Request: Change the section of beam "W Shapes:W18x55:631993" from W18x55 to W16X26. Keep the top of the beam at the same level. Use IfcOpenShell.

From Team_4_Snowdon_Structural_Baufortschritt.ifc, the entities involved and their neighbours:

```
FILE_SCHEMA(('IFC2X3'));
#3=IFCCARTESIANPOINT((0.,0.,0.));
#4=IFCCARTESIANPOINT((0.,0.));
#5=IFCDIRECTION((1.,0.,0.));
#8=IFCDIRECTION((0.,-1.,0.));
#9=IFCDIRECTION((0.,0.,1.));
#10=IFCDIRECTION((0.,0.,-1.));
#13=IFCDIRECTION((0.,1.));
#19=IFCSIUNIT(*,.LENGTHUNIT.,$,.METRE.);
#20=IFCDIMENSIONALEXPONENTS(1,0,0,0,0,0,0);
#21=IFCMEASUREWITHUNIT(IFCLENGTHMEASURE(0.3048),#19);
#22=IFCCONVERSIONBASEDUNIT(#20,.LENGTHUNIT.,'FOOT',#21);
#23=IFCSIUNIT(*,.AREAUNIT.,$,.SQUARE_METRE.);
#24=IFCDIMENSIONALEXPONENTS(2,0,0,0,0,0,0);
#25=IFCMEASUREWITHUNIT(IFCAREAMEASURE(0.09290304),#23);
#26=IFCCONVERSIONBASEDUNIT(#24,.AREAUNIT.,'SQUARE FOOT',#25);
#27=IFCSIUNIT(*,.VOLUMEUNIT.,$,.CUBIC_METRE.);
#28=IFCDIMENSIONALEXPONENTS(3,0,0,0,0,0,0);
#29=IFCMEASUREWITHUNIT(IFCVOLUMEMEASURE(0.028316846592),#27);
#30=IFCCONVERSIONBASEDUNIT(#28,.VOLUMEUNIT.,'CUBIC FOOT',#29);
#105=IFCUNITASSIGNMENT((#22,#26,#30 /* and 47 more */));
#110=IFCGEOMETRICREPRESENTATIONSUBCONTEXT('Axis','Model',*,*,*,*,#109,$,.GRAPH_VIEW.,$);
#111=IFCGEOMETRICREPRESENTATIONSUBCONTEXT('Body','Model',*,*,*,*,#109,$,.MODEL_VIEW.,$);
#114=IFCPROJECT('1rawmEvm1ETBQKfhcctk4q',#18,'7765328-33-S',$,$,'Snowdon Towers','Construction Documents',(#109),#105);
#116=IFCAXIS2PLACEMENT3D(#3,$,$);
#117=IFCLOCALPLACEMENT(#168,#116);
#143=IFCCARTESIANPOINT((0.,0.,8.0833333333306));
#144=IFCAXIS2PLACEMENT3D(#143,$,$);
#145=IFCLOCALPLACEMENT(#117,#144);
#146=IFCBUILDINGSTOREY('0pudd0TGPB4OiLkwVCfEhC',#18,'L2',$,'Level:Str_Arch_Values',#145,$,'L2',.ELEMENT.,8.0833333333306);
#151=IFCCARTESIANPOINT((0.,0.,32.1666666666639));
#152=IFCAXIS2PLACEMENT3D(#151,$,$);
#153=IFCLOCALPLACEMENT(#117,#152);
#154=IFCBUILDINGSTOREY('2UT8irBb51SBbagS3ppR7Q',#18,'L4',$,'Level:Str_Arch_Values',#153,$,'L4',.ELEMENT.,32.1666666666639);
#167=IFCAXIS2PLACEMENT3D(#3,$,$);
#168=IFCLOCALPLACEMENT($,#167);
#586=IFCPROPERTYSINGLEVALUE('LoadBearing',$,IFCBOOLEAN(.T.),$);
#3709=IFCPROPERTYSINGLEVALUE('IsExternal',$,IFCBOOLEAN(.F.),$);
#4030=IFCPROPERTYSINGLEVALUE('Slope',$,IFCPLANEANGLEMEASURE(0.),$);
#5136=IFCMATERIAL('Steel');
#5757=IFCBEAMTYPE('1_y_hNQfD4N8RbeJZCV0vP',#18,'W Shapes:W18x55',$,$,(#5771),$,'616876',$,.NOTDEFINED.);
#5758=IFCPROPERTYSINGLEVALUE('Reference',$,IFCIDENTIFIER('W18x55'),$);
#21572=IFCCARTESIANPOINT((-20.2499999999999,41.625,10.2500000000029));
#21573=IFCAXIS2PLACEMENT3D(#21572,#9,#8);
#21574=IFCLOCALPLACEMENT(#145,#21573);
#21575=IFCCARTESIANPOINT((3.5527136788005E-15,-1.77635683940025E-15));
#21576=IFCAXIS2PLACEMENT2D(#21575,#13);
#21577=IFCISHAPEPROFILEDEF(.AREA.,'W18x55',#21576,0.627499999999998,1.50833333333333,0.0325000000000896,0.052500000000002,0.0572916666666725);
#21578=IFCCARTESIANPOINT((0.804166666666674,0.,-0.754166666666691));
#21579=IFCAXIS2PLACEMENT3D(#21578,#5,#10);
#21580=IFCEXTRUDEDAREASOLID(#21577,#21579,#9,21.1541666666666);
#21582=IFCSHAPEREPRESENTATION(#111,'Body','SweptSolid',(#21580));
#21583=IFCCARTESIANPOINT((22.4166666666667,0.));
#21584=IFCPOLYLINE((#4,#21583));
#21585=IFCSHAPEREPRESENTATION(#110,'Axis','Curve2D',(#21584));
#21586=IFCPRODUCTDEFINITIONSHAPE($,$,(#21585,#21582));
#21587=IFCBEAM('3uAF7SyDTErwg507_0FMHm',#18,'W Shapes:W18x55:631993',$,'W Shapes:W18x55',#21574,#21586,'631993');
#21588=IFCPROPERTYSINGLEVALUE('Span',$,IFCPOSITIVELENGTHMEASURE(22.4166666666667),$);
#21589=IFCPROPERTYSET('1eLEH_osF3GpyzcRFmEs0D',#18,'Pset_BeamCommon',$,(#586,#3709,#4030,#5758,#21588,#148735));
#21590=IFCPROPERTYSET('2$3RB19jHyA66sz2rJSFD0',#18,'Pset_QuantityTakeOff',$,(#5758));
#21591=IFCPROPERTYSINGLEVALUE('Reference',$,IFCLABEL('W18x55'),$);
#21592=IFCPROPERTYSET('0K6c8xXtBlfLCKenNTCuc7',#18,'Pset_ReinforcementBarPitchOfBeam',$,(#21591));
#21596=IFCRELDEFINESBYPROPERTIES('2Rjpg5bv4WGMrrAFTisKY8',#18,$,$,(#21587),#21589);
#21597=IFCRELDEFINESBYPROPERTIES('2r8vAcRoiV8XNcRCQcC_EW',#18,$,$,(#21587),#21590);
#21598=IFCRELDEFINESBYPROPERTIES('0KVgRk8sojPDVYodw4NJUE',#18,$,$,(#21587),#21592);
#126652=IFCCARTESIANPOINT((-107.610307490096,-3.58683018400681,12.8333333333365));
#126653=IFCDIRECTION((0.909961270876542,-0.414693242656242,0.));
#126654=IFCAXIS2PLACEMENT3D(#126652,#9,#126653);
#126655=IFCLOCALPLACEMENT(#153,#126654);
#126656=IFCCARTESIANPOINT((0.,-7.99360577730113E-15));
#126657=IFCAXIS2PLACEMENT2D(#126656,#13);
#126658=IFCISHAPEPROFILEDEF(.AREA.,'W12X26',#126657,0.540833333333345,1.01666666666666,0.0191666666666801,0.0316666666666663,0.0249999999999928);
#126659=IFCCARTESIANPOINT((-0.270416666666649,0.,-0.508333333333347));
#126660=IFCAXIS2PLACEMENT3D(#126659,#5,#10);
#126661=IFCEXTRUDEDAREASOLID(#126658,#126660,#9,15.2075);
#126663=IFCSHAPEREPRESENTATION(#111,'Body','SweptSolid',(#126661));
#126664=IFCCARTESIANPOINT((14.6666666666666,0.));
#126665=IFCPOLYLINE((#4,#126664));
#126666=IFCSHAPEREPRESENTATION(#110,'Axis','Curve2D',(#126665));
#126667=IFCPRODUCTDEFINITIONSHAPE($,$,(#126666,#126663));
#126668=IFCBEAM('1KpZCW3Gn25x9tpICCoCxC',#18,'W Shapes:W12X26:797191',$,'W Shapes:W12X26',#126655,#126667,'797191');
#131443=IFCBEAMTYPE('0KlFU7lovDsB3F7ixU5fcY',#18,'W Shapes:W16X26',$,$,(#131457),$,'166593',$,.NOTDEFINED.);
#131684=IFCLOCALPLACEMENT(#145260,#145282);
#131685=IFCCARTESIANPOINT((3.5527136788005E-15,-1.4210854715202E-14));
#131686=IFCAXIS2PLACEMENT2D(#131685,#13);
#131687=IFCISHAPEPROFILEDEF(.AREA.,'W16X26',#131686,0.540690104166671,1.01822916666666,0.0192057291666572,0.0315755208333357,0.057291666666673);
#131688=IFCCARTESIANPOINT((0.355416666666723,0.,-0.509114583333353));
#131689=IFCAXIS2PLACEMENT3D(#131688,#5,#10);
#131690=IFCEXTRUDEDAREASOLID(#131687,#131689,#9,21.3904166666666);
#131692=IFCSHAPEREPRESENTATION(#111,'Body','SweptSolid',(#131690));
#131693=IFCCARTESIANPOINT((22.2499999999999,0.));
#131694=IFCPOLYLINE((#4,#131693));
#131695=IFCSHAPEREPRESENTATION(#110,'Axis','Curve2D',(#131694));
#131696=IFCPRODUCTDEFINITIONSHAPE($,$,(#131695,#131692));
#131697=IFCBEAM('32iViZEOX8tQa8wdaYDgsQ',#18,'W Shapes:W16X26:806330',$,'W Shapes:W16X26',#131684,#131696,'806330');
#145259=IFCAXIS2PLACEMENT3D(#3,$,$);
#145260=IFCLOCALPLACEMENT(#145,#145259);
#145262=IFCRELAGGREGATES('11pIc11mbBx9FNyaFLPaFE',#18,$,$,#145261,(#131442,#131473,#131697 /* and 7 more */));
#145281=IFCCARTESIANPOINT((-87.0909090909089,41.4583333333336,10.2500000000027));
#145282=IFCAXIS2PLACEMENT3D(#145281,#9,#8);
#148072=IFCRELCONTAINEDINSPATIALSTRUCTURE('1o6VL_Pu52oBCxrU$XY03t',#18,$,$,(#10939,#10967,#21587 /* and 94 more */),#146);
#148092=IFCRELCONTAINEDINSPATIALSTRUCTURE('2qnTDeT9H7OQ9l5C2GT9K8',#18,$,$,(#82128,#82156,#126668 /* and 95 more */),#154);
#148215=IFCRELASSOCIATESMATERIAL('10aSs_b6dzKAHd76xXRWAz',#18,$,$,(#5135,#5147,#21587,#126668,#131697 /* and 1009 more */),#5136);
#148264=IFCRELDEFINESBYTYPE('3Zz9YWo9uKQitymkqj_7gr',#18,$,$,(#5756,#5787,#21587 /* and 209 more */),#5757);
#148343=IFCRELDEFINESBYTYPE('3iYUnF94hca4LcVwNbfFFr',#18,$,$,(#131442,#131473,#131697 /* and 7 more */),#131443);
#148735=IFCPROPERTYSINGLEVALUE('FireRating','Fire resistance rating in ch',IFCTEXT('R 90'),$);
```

```python
import ifcopenshell
import ifcopenshell.api.pset
import ifcopenshell.api.type
import ifcopenshell.util.element
import ifcopenshell.util.representation

model = ifcopenshell.open("Team_4_Snowdon_Structural_Baufortschritt.ifc")

member = model.by_guid("3uAF7SyDTErwg507_0FMHm")
source = next(p for p in model.by_type("IfcIShapeProfileDef") if p.ProfileName == "W16X26")

body = ifcopenshell.util.representation.get_representation(member, "Model", "Body")
solid = body.Items[0]
old_profile = solid.SweptArea

# Copy the section's sizes but keep this member's own profile position.
profile = ifcopenshell.util.element.copy(model, source)
# Profiles are centred, so shift by half the change in depth to hold the top.
shift = (old_profile.OverallDepth - profile.OverallDepth) / 2
x, y = old_profile.Position.Location.Coordinates
up = (-1.0, 0.0)  # upwards, in the solid's own plane
location = model.createIfcCartesianPoint((x + up[0] * shift, y + up[1] * shift))
profile.Position = model.createIfcAxis2Placement2D(location, old_profile.Position.RefDirection)
solid.SweptArea = profile
if not model.get_total_inverses(old_profile):
    ifcopenshell.util.element.remove_deep2(model, old_profile)

new_type = model.by_id(131443)
ifcopenshell.api.type.assign_type(
    model, related_objects=[member], relating_type=new_type, should_map_representations=False
)
member.Name = member.Name.replace("W18x55", "W16X26")
member.ObjectType = "W Shapes:W16X26"
pset = model.by_id(ifcopenshell.util.element.get_pset(member, "Pset_BeamCommon", should_inherit=False)["id"])
ifcopenshell.api.pset.edit_pset(model, pset=pset, properties={"Reference": "W16X26"})
pset = model.by_id(ifcopenshell.util.element.get_pset(member, "Pset_QuantityTakeOff", should_inherit=False)["id"])
ifcopenshell.api.pset.edit_pset(model, pset=pset, properties={"Reference": "W16X26"})
pset = model.by_id(ifcopenshell.util.element.get_pset(member, "Pset_ReinforcementBarPitchOfBeam", should_inherit=False)["id"])
ifcopenshell.api.pset.edit_pset(model, pset=pset, properties={"Reference": "W16X26"})

print(solid.SweptArea)

model.write("Team_4_Snowdon_Structural_Baufortschritt-out.ifc")
```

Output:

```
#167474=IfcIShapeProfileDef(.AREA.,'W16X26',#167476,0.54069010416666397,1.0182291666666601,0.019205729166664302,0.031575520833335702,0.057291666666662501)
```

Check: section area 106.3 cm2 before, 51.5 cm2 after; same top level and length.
